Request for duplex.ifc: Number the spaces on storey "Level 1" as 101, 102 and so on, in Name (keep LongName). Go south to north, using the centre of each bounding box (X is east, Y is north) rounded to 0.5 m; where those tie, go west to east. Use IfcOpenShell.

First a look at what the model holds.

```python
import ifcopenshell
import ifcopenshell.util.element
import ifcopenshell.util.placement

model = ifcopenshell.open("duplex.ifc")
print(model.schema)
storey = next(s for s in model.by_type("IfcBuildingStorey") if s.Name == "Level 1")
spaces = [e for e in ifcopenshell.util.element.get_decomposition(storey) if e.is_a("IfcSpace")]
for e in sorted(spaces, key=lambda e: e.id()):
    origin = ifcopenshell.util.placement.get_local_placement(e.ObjectPlacement)[:3, 3]
    print(e.id(), e.Name, e.LongName, origin.round(2) + 0.0, sep=" | ")
```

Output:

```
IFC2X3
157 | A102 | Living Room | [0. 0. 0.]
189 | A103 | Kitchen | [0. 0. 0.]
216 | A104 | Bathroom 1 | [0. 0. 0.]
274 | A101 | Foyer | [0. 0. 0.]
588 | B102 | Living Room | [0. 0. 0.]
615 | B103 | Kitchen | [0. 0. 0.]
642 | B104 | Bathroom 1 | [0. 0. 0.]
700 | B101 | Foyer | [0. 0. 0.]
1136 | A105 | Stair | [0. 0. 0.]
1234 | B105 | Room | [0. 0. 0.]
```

```python
import ifcopenshell
import ifcopenshell.geom
import ifcopenshell.util.element
import ifcopenshell.util.shape

model = ifcopenshell.open("duplex.ifc")
settings = ifcopenshell.geom.settings()
settings.set("use-world-coords", True)


def centre(element):
    shape = ifcopenshell.geom.create_shape(settings, element)
    return ifcopenshell.util.shape.get_bbox_centroid(shape.geometry)


storey = next(s for s in model.by_type("IfcBuildingStorey") if s.Name == "Level 1")
spaces = [e for e in ifcopenshell.util.element.get_decomposition(storey) if e.is_a("IfcSpace")]

# Insertion points can sit at a corner or the storey origin, so sort by the geometry (in metres).
centres = {e: centre(e) for e in spaces}
spaces.sort(key=lambda e: (round(centres[e][1] / 0.5), centres[e][0]))

for i, e in enumerate(spaces, start=1):
    number = f"1{i:02d}"
    e.Name = number
    print(e.id(), number)

model.write("duplex-out.ifc")
```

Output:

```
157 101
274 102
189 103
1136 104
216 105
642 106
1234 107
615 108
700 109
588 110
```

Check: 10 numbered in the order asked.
